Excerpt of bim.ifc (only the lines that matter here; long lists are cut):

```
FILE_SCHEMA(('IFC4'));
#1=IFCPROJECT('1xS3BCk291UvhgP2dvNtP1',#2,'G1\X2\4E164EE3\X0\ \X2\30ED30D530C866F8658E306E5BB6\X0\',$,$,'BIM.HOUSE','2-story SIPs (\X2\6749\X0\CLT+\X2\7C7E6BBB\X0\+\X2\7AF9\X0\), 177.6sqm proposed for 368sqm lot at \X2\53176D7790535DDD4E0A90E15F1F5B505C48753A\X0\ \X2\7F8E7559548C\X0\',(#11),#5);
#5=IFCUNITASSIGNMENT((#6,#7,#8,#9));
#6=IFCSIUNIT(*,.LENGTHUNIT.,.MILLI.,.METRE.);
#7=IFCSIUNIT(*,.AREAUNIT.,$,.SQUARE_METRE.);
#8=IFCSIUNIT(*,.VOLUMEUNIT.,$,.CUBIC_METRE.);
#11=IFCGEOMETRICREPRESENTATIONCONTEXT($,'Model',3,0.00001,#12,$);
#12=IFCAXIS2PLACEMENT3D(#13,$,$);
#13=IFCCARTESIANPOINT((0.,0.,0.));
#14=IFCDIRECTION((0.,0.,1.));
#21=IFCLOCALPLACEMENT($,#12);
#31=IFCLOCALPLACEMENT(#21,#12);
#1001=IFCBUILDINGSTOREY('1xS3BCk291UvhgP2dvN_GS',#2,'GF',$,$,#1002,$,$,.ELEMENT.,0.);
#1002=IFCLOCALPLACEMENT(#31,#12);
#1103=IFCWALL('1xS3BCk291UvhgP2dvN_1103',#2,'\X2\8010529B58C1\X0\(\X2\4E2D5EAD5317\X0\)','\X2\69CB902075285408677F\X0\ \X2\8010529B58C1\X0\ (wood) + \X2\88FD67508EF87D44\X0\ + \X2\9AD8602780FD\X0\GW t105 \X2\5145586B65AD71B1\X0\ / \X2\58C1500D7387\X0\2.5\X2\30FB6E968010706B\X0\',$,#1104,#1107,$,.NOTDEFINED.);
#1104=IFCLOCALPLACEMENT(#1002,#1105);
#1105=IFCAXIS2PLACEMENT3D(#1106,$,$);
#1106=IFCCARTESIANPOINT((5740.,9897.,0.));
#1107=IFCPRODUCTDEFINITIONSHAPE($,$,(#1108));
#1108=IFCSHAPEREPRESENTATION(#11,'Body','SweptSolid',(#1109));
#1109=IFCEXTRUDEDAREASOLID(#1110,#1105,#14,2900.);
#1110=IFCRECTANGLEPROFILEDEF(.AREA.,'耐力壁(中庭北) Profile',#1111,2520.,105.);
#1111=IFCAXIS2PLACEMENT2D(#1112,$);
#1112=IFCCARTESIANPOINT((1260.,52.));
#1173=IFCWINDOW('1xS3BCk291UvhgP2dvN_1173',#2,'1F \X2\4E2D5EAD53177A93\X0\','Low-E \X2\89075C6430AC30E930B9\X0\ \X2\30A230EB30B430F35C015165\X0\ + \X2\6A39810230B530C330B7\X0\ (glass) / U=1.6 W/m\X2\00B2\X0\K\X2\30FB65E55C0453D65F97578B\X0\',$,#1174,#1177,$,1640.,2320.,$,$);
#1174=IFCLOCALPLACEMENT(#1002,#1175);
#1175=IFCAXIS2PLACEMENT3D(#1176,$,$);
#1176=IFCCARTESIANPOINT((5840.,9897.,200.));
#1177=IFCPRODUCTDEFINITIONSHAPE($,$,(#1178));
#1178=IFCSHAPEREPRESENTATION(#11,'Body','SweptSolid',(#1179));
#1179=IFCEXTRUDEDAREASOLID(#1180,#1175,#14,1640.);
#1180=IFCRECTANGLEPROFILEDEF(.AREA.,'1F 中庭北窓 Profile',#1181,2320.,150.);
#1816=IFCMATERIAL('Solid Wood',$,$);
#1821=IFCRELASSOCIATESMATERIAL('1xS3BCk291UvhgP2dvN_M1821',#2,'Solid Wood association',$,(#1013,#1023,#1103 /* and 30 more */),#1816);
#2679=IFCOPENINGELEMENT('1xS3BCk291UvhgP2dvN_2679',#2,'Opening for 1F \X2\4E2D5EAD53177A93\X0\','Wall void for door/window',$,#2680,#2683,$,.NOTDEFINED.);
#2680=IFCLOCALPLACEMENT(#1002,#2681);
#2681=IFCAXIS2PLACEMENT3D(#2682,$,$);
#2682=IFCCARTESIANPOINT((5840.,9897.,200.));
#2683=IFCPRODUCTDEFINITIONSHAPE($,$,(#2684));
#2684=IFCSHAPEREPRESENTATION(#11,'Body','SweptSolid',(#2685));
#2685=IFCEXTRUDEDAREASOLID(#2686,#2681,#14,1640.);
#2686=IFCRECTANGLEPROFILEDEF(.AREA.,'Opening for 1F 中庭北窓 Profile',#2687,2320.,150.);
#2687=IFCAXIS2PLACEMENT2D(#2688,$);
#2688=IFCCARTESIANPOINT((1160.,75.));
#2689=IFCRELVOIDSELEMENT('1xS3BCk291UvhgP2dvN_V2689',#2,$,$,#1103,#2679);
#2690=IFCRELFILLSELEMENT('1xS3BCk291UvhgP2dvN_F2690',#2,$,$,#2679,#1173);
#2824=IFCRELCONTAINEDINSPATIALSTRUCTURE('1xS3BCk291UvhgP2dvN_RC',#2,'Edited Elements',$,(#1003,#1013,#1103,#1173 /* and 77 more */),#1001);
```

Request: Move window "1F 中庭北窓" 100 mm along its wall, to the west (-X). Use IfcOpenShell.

```python
import ifcopenshell
import ifcopenshell.api.geometry
import ifcopenshell.util.placement

model = ifcopenshell.open("bim.ifc")

window = model.by_guid("1xS3BCk291UvhgP2dvN_1173")
opening = window.FillsVoids[0].RelatingOpeningElement
wall = opening.VoidsElements[0].RelatingBuildingElement

wall_matrix = ifcopenshell.util.placement.get_local_placement(wall.ObjectPlacement)
shift = wall_matrix[:3, 0] * -100.0
before = ifcopenshell.util.placement.get_local_placement(window.ObjectPlacement)[:3, 3].copy()

# The window is not placed relative to its opening, so move both.
for product in (opening, window):
    matrix = ifcopenshell.util.placement.get_local_placement(product.ObjectPlacement)
    matrix[:3, 3] += shift
    ifcopenshell.api.geometry.edit_object_placement(model, product=product, matrix=matrix, is_si=False)

after = ifcopenshell.util.placement.get_local_placement(window.ObjectPlacement)[:3, 3]
print("window moved by", (after - before).round(3) + 0.0)

model.write("bim_rev.ifc")
```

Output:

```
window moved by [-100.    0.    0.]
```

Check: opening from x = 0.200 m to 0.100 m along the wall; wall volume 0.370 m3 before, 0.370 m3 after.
